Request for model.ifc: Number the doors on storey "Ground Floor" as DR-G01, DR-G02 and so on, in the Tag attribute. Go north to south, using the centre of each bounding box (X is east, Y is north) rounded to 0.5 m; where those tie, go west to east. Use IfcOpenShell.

First a look at what the model holds.

```python
import ifcopenshell
import ifcopenshell.util.element
import ifcopenshell.util.placement

model = ifcopenshell.open("model.ifc")
print(model.schema)
storey = next(s for s in model.by_type("IfcBuildingStorey") if s.Name == "Ground Floor")
doors = [e for e in ifcopenshell.util.element.get_decomposition(storey) if e.is_a("IfcDoor")]
for e in sorted(doors, key=lambda e: e.id()):
    origin = ifcopenshell.util.placement.get_local_placement(e.ObjectPlacement)[:3, 3]
    print(e.id(), e.Tag, e.Name, origin.round(2) + 0.0, sep=" | ")
```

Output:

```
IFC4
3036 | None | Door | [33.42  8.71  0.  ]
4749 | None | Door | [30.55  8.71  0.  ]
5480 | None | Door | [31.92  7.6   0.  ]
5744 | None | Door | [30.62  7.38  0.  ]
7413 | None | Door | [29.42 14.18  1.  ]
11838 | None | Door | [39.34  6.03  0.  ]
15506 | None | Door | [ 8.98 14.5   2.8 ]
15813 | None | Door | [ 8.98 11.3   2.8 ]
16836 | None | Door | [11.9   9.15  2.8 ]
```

```python
import ifcopenshell
import ifcopenshell.geom
import ifcopenshell.util.element
import ifcopenshell.util.shape

model = ifcopenshell.open("model.ifc")
settings = ifcopenshell.geom.settings()
settings.set("use-world-coords", True)


def centre(element):
    shape = ifcopenshell.geom.create_shape(settings, element)
    return ifcopenshell.util.shape.get_bbox_centroid(shape.geometry)


storey = next(s for s in model.by_type("IfcBuildingStorey") if s.Name == "Ground Floor")
doors = [e for e in ifcopenshell.util.element.get_decomposition(storey) if e.is_a("IfcDoor")]

# Insertion points can sit at a corner or the storey origin, so sort by the geometry (in metres).
centres = {e: centre(e) for e in doors}
doors.sort(key=lambda e: (-round(centres[e][1] / 0.5), centres[e][0]))

for i, e in enumerate(doors, start=1):
    number = f"DR-G{i:02d}"
    e.Tag = number
    print(e.id(), number)

model.write("model_rev.ifc")
```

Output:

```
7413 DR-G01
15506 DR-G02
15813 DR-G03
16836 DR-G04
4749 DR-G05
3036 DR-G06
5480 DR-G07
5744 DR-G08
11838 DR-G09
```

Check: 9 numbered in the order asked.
